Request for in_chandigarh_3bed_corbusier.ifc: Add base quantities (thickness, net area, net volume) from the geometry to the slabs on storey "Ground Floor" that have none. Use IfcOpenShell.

First a look at what the model holds.

```python
import ifcopenshell
import ifcopenshell.util.element
import ifcopenshell.util.unit

model = ifcopenshell.open("in_chandigarh_3bed_corbusier.ifc")
print(model.schema)
for unit_type in ("LENGTHUNIT", "AREAUNIT", "VOLUMEUNIT"):
    print(unit_type, ifcopenshell.util.unit.calculate_unit_scale(model, unit_type))
storey = next(s for s in model.by_type("IfcBuildingStorey") if s.Name == "Ground Floor")
slabs = [e for e in ifcopenshell.util.element.get_decomposition(storey) if e.is_a("IfcSlab")]
for e in sorted(slabs, key=lambda e: e.id()):
    print(e.id(), e.is_a(), e.Name, list(ifcopenshell.util.element.get_psets(e, qtos_only=True)), sep=" | ")
```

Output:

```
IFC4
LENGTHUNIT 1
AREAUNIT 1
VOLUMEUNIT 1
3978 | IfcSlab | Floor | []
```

```python
import ifcopenshell
import ifcopenshell.api.pset
import ifcopenshell.geom
import ifcopenshell.util.element
import ifcopenshell.util.shape
import ifcopenshell.util.unit

model = ifcopenshell.open("in_chandigarh_3bed_corbusier.ifc")
unit_scale = ifcopenshell.util.unit.calculate_unit_scale(model)
area_scale = ifcopenshell.util.unit.calculate_unit_scale(model, "AREAUNIT")
volume_scale = ifcopenshell.util.unit.calculate_unit_scale(model, "VOLUMEUNIT")
settings = ifcopenshell.geom.settings()

storey = next(s for s in model.by_type("IfcBuildingStorey") if s.Name == "Ground Floor")
slabs = [e for e in ifcopenshell.util.element.get_decomposition(storey) if e.is_a("IfcSlab")]

for e in sorted(slabs, key=lambda e: e.id()):
    if ifcopenshell.util.element.get_psets(e, qtos_only=True, should_inherit=False):
        continue
    # Geometry comes back in metres, in the element's own axes.
    shape = ifcopenshell.geom.create_shape(settings, e)
    values = {
        "Width": ifcopenshell.util.shape.get_z(shape.geometry) / unit_scale,
        "NetArea": ifcopenshell.util.shape.get_footprint_area(shape.geometry) / area_scale,
        "NetVolume": ifcopenshell.util.shape.get_volume(shape.geometry) / volume_scale,
    }
    qto = ifcopenshell.api.pset.add_qto(model, product=e, name="Qto_SlabBaseQuantities")
    ifcopenshell.api.pset.edit_qto(model, qto=qto, properties=values)
    print(e.id(), {k: round(v, 3) for k, v in values.items()})

model.write("in_chandigarh_3bed_corbusier_rev.ifc")
```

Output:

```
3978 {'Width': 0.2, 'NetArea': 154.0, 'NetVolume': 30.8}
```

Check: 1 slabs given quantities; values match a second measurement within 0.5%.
